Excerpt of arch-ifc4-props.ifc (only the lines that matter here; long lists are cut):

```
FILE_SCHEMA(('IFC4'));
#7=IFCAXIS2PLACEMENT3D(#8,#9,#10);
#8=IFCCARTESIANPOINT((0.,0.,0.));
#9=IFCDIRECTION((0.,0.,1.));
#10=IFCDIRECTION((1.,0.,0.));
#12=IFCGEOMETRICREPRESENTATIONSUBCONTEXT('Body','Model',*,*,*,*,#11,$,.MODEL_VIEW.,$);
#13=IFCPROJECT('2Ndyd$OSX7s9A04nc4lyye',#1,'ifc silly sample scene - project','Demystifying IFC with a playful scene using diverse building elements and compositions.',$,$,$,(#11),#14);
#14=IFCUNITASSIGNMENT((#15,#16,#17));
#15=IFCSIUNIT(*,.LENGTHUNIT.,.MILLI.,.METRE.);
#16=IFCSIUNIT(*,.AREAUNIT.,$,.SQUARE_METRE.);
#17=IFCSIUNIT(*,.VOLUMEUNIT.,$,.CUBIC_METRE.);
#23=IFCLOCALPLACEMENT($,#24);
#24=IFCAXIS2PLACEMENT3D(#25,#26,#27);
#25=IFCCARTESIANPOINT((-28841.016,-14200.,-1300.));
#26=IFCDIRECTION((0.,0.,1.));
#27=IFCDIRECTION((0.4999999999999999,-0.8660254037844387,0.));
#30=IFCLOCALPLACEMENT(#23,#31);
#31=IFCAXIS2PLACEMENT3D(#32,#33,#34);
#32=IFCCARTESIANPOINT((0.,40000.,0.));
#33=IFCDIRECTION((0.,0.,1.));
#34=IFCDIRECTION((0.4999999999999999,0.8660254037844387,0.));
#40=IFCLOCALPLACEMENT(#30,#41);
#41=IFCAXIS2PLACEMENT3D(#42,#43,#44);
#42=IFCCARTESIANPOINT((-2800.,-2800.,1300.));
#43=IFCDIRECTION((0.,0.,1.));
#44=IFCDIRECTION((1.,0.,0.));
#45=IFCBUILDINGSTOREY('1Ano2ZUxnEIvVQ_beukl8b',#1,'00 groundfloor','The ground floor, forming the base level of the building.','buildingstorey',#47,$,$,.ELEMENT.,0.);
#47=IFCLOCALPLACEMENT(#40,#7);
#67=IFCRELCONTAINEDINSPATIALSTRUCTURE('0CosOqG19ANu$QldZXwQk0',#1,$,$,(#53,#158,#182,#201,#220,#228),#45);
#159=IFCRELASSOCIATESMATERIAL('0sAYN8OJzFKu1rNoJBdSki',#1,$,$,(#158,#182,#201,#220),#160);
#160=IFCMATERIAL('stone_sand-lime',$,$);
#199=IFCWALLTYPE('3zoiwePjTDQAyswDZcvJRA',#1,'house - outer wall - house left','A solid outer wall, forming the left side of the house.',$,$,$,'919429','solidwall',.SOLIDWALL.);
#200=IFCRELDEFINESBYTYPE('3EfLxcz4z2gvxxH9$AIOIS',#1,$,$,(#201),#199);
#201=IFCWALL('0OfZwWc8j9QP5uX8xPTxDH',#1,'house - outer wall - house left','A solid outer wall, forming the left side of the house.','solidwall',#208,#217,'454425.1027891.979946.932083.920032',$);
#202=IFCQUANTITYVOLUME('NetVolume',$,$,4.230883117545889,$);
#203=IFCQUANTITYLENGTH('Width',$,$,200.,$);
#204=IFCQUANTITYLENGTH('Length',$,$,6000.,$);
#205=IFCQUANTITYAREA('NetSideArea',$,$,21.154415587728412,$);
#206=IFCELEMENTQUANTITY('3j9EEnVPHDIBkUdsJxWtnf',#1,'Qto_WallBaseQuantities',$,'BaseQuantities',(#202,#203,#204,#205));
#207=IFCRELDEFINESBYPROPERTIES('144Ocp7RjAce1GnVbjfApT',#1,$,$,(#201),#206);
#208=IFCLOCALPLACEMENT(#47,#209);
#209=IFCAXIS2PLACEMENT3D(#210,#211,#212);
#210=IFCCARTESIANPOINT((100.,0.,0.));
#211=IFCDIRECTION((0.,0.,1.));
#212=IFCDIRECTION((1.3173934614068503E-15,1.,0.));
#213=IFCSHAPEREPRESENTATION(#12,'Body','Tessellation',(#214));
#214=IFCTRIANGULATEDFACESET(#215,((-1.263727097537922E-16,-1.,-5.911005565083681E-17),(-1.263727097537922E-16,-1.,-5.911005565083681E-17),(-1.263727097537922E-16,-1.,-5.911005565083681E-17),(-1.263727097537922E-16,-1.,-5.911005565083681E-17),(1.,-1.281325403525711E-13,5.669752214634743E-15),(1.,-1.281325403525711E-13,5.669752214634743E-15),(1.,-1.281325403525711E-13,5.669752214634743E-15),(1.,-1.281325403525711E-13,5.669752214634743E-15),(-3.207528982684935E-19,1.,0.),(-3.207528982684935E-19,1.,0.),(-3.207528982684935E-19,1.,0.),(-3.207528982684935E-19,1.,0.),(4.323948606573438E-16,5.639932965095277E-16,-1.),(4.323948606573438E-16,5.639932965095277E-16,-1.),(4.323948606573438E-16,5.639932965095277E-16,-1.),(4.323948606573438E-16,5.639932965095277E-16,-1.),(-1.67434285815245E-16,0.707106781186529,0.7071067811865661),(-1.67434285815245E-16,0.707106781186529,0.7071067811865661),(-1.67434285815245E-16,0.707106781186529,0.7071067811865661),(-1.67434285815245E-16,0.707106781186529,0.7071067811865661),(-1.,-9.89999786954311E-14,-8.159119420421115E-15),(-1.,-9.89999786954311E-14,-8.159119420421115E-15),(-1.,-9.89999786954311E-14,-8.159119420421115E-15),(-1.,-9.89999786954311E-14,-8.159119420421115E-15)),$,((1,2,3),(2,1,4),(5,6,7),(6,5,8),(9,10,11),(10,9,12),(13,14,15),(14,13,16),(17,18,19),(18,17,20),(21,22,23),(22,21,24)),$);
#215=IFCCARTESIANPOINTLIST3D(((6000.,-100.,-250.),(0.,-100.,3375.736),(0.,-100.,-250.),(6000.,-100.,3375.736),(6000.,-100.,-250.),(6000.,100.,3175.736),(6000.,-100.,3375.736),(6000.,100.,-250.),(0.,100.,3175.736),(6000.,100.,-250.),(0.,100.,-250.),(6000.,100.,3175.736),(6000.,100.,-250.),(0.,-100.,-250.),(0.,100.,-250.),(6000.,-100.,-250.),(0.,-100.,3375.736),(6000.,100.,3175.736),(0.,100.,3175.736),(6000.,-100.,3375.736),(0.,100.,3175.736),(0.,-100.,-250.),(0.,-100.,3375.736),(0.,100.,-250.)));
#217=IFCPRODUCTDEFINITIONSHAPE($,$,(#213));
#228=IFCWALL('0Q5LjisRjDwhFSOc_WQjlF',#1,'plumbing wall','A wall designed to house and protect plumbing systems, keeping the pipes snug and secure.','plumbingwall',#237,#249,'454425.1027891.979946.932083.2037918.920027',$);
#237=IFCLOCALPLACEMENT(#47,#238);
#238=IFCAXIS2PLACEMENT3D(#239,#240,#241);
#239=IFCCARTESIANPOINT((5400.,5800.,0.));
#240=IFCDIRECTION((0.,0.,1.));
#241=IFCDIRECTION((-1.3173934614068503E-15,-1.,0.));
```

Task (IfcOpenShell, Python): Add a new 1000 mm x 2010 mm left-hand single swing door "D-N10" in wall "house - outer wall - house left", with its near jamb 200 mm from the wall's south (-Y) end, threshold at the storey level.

```python
import numpy as np
import ifcopenshell
import ifcopenshell.api.feature
import ifcopenshell.api.geometry
import ifcopenshell.api.pset
import ifcopenshell.api.root
import ifcopenshell.api.spatial
import ifcopenshell.geom
import ifcopenshell.util.element
import ifcopenshell.util.placement
import ifcopenshell.util.representation
import ifcopenshell.util.shape
import ifcopenshell.util.unit

model = ifcopenshell.open("arch-ifc4-props.ifc")
unit_scale = ifcopenshell.util.unit.calculate_unit_scale(model)
area_scale = ifcopenshell.util.unit.calculate_unit_scale(model, "AREAUNIT")
volume_scale = ifcopenshell.util.unit.calculate_unit_scale(model, "VOLUMEUNIT")
settings = ifcopenshell.geom.settings()


def volume(element):
    """Net volume in cubic metres, openings subtracted."""
    shape = ifcopenshell.geom.create_shape(settings, element)
    return ifcopenshell.util.shape.get_volume(shape.geometry)


wall = model.by_guid("0OfZwWc8j9QP5uX8xPTxDH")
storey = ifcopenshell.util.element.get_container(wall, ifc_class="IfcBuildingStorey")
context = ifcopenshell.util.representation.get_context(model, "Model", "Body", "MODEL_VIEW")
before = volume(wall)

width, height, from_end, sill = 1, 2.01, 0.2, 0.0  # metres

# The wall runs along its own X axis, and the end named is its -X end.
wall_shape = ifcopenshell.geom.create_shape(settings, wall)
x, y, z = ifcopenshell.util.shape.get_vertices(wall_shape.geometry).T
start = x.min() + from_end
face, thickness = float(y.min()), float(y.max() - y.min())
wall_matrix = ifcopenshell.util.placement.get_local_placement(wall.ObjectPlacement)
level = ifcopenshell.util.placement.get_local_placement(storey.ObjectPlacement)[2, 3]


def in_wall(x, y):
    """Placement at x, y metres in the wall's axes, at sill height."""
    matrix = wall_matrix.copy()
    matrix[:, 3] = wall_matrix @ np.array([x / unit_scale, y / unit_scale, 0.0, 1.0])
    matrix[2, 3] = level + sill / unit_scale
    return matrix


# Opening: a box that overshoots both wall faces by 50 mm.
opening = ifcopenshell.api.root.create_entity(model, ifc_class="IfcOpeningElement", predefined_type="OPENING")
box = ifcopenshell.api.geometry.add_wall_representation(
    model, context=context, length=width, height=height, thickness=thickness + 0.1
)
ifcopenshell.api.geometry.assign_representation(model, product=opening, representation=box)
ifcopenshell.api.geometry.edit_object_placement(model, product=opening, matrix=in_wall(start, face - 0.05), is_si=False)
ifcopenshell.api.feature.add_feature(model, feature=opening, element=wall)

door = ifcopenshell.api.root.create_entity(model, ifc_class="IfcDoor", name="D-N10", predefined_type="DOOR")
door.OverallWidth, door.OverallHeight = width / unit_scale, height / unit_scale
door.OperationType = "SINGLE_SWING_LEFT"
body = ifcopenshell.api.geometry.add_door_representation(
    model,
    context=context,
    overall_width=door.OverallWidth,
    overall_height=door.OverallHeight,
    operation_type="SINGLE_SWING_LEFT",
    lining_properties={"LiningDepth": thickness / unit_scale, "ThresholdDepth": thickness / unit_scale},
)
ifcopenshell.api.geometry.assign_representation(model, product=door, representation=body)
ifcopenshell.api.spatial.assign_container(model, products=[door], relating_structure=storey)
ifcopenshell.api.feature.add_filling(model, opening=opening, element=door)

# The lining spans the wall, so the door starts at the wall face.
ifcopenshell.api.geometry.edit_object_placement(model, product=door, matrix=in_wall(start, face), is_si=False)

after = volume(wall)

# Update the wall's stored quantities.
qto = model.by_id(ifcopenshell.util.element.get_pset(wall, "Qto_WallBaseQuantities", should_inherit=False)["id"])
ifcopenshell.api.pset.edit_qto(model, qto=qto, properties={
    "NetVolume": after / volume_scale,
    "NetSideArea": after / thickness / area_scale,
})

print(f"wall volume {before:.3f} -> {after:.3f} m3")

model.write("arch-ifc4-props_rev.ifc")
```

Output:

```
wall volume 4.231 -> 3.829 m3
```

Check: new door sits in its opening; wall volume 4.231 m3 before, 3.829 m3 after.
